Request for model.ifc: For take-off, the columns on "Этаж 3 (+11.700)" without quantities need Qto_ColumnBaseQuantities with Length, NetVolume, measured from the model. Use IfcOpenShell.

First a look at what the model holds.

```python
import ifcopenshell
import ifcopenshell.util.element
import ifcopenshell.util.unit

model = ifcopenshell.open("model.ifc")
print(model.schema)
for unit_type in ("LENGTHUNIT", "AREAUNIT", "VOLUMEUNIT"):
    print(unit_type, ifcopenshell.util.unit.calculate_unit_scale(model, unit_type))
storey = next(s for s in model.by_type("IfcBuildingStorey") if s.Name == "Этаж 3 (+11.700)")
columns = [e for e in ifcopenshell.util.element.get_decomposition(storey) if e.is_a("IfcColumn")]
for e in sorted(columns, key=lambda e: e.id()):
    print(e.id(), e.is_a(), e.Name, list(ifcopenshell.util.element.get_psets(e, qtos_only=True)), sep=" | ")
```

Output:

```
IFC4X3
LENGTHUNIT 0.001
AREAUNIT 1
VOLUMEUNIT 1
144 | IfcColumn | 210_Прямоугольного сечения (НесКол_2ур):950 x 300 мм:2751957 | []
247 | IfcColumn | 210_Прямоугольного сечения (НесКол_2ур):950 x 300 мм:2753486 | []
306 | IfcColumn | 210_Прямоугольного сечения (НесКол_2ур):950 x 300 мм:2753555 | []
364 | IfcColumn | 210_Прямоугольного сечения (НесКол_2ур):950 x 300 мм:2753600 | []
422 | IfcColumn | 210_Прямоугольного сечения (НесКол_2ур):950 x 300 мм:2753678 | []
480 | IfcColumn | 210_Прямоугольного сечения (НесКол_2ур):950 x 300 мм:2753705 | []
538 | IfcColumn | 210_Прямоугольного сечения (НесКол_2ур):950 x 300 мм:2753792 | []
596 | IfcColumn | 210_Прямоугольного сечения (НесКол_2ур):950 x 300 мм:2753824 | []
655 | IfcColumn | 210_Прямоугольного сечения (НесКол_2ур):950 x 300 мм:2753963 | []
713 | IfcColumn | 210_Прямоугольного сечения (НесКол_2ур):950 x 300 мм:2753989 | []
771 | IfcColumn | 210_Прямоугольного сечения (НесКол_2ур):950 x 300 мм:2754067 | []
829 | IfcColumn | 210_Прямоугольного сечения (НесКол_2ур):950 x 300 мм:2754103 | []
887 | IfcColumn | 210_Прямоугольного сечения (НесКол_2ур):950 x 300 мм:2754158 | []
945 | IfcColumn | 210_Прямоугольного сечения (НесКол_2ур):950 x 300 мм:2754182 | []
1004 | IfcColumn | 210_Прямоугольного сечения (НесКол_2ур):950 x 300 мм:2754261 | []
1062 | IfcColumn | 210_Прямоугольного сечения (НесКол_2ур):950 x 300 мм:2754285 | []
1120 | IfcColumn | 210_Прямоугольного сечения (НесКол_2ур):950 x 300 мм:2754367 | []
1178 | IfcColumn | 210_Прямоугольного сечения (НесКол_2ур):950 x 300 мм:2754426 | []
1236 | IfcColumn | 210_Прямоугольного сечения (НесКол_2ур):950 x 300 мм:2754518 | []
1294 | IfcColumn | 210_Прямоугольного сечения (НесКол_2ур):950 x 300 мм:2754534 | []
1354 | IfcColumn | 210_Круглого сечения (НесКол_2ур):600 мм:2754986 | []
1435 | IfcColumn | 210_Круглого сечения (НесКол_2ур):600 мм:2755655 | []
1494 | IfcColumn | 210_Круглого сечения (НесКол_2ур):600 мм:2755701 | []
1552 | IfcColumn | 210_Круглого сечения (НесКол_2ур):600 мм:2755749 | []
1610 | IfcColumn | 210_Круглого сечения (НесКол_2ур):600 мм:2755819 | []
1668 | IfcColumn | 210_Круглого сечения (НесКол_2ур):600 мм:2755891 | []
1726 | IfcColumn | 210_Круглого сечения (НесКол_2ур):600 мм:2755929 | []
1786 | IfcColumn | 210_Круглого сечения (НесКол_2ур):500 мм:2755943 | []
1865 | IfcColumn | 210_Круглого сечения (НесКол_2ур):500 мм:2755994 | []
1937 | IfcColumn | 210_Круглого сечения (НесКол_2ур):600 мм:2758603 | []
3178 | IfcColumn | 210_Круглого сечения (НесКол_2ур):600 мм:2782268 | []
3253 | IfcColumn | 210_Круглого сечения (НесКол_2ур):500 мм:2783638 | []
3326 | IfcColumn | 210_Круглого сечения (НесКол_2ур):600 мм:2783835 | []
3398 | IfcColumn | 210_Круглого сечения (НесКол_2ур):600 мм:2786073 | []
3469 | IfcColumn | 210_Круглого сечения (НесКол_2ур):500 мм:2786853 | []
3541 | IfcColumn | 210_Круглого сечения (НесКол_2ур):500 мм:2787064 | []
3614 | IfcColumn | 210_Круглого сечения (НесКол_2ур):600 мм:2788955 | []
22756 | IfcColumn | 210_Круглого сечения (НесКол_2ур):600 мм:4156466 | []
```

```python
import ifcopenshell
import ifcopenshell.api.pset
import ifcopenshell.geom
import ifcopenshell.util.element
import ifcopenshell.util.shape
import ifcopenshell.util.unit

model = ifcopenshell.open("model.ifc")
unit_scale = ifcopenshell.util.unit.calculate_unit_scale(model)
volume_scale = ifcopenshell.util.unit.calculate_unit_scale(model, "VOLUMEUNIT")
settings = ifcopenshell.geom.settings()

storey = next(s for s in model.by_type("IfcBuildingStorey") if s.Name == "Этаж 3 (+11.700)")
columns = [e for e in ifcopenshell.util.element.get_decomposition(storey) if e.is_a("IfcColumn")]

for e in sorted(columns, key=lambda e: e.id()):
    if ifcopenshell.util.element.get_psets(e, qtos_only=True, should_inherit=False):
        continue
    # Geometry comes back in metres, in the element's own axes.
    shape = ifcopenshell.geom.create_shape(settings, e)
    values = {
        "Length": ifcopenshell.util.shape.get_z(shape.geometry) / unit_scale,
        "NetVolume": ifcopenshell.util.shape.get_volume(shape.geometry) / volume_scale,
    }
    qto = ifcopenshell.api.pset.add_qto(model, product=e, name="Qto_ColumnBaseQuantities")
    ifcopenshell.api.pset.edit_qto(model, qto=qto, properties=values)
    print(e.id(), {k: round(v, 3) for k, v in values.items()})

model.write("model_rev.ifc")
```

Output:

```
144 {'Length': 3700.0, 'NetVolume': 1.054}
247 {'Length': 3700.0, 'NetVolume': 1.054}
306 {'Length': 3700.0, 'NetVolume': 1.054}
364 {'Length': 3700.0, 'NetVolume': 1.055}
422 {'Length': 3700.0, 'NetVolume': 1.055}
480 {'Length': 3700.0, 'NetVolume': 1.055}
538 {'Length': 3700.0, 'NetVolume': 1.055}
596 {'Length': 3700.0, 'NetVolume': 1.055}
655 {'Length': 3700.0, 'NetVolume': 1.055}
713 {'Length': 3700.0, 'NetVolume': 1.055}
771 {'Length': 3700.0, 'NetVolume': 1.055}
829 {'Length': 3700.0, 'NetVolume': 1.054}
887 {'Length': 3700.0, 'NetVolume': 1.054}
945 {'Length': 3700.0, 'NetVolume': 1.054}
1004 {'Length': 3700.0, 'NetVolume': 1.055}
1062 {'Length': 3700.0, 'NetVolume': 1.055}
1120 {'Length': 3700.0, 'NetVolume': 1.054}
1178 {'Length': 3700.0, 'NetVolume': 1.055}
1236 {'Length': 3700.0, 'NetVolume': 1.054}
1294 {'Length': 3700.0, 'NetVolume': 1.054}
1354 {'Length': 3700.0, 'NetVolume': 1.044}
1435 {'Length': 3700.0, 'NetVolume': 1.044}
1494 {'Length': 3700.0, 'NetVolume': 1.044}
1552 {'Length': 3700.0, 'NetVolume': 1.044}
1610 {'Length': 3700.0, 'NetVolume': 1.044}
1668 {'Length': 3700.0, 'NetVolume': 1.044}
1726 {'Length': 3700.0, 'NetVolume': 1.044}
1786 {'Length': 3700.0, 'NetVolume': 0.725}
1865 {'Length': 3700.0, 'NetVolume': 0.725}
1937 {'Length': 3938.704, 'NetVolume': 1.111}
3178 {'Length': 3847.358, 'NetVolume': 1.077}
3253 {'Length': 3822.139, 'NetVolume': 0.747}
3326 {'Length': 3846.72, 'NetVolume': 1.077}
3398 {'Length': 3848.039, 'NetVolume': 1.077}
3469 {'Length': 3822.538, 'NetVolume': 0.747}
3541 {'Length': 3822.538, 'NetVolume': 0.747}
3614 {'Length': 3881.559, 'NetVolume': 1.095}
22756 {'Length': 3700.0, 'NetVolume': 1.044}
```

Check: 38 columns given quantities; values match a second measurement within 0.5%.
